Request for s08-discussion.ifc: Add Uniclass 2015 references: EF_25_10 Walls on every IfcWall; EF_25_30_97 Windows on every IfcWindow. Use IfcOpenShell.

First a look at what the model holds.

```python
import ifcopenshell

model = ifcopenshell.open("s08-discussion.ifc")
print(model.schema)
print("classifications:", [c.Name for c in model.by_type("IfcClassification")])
for ifc_class in ("IfcDoor", "IfcRoof", "IfcStair", "IfcWall", "IfcWindow"):
    print(ifc_class, len(model.by_type(ifc_class)))
```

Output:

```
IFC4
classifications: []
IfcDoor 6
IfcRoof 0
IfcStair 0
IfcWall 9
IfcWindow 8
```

```python
import ifcopenshell
import ifcopenshell.api.classification

model = ifcopenshell.open("s08-discussion.ifc")

system = ifcopenshell.api.classification.add_classification(model, classification="Uniclass 2015")

codes = {
    "IfcWall": ("EF_25_10", "Walls"),
    "IfcWindow": ("EF_25_30_97", "Windows"),
}
for ifc_class, (code, name) in codes.items():
    products = model.by_type(ifc_class)
    ifcopenshell.api.classification.add_reference(
        model, products=products, classification=system, identification=code, name=name
    )
    print(code, len(products))

model.write("s08-discussion_rev.ifc")
```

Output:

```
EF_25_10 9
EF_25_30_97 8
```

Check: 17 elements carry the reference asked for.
